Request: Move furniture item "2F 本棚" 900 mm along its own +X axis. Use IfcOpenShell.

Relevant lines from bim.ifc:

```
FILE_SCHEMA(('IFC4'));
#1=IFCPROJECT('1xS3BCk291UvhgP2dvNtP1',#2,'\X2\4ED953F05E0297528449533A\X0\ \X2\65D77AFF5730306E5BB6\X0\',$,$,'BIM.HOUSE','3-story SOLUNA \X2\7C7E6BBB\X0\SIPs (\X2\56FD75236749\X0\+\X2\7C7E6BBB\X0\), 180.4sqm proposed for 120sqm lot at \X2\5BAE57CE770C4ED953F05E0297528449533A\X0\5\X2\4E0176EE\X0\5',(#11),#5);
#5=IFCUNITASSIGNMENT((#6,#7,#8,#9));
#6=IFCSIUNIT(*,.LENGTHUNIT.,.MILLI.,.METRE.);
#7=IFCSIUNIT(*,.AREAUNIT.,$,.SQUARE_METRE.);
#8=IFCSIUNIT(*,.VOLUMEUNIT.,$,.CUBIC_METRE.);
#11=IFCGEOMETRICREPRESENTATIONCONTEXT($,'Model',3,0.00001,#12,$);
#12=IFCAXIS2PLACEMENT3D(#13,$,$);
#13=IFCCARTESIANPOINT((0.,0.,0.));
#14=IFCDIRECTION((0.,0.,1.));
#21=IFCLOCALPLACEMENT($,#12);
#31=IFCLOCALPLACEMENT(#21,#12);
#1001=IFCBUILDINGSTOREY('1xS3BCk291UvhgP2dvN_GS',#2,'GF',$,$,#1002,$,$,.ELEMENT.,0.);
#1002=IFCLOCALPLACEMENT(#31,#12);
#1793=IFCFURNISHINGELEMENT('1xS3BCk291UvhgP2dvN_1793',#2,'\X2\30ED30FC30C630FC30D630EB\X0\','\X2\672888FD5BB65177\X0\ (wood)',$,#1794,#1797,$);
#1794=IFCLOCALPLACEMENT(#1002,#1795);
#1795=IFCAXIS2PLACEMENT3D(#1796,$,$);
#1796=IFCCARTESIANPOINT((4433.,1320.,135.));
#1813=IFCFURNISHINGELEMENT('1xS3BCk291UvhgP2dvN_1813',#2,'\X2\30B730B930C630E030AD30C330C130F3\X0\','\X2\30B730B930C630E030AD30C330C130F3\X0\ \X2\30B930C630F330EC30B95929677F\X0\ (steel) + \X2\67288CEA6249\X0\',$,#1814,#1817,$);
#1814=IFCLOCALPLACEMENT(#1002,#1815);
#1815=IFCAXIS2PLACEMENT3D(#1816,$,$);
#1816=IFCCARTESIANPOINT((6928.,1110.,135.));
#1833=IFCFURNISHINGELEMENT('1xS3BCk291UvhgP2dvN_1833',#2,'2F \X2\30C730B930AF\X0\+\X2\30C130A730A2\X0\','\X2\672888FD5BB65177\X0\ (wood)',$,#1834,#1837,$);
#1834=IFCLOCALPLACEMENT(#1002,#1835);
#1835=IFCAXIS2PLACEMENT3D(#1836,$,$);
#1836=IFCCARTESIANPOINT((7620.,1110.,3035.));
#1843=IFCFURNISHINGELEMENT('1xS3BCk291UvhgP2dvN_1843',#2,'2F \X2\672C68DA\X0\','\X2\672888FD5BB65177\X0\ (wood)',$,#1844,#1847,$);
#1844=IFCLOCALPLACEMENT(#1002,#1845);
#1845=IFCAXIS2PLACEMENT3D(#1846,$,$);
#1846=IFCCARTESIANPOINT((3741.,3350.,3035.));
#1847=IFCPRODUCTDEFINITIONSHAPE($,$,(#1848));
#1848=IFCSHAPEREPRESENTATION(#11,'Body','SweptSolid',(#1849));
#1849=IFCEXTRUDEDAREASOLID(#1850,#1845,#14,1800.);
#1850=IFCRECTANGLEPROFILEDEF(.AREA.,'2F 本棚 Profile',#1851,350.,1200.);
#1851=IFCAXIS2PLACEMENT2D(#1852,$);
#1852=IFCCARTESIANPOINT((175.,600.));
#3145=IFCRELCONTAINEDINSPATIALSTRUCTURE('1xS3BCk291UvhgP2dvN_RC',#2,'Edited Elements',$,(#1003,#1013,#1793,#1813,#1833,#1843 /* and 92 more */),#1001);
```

```python
import ifcopenshell
import ifcopenshell.api.geometry
import ifcopenshell.util.placement

model = ifcopenshell.open("bim.ifc")

item = model.by_guid("1xS3BCk291UvhgP2dvN_1843")
matrix = ifcopenshell.util.placement.get_local_placement(item.ObjectPlacement)
matrix[:3, 3] += matrix[:3, 0] * 900.0
ifcopenshell.api.geometry.edit_object_placement(model, product=item, matrix=matrix, is_si=False)

print(ifcopenshell.util.placement.get_local_placement(item.ObjectPlacement).round(3) + 0.0)

model.write("bim_v2.ifc")
```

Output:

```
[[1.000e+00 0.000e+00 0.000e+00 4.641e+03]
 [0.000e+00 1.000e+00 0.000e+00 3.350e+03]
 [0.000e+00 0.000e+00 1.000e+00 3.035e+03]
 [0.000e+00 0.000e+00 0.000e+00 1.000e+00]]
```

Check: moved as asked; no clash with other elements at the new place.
